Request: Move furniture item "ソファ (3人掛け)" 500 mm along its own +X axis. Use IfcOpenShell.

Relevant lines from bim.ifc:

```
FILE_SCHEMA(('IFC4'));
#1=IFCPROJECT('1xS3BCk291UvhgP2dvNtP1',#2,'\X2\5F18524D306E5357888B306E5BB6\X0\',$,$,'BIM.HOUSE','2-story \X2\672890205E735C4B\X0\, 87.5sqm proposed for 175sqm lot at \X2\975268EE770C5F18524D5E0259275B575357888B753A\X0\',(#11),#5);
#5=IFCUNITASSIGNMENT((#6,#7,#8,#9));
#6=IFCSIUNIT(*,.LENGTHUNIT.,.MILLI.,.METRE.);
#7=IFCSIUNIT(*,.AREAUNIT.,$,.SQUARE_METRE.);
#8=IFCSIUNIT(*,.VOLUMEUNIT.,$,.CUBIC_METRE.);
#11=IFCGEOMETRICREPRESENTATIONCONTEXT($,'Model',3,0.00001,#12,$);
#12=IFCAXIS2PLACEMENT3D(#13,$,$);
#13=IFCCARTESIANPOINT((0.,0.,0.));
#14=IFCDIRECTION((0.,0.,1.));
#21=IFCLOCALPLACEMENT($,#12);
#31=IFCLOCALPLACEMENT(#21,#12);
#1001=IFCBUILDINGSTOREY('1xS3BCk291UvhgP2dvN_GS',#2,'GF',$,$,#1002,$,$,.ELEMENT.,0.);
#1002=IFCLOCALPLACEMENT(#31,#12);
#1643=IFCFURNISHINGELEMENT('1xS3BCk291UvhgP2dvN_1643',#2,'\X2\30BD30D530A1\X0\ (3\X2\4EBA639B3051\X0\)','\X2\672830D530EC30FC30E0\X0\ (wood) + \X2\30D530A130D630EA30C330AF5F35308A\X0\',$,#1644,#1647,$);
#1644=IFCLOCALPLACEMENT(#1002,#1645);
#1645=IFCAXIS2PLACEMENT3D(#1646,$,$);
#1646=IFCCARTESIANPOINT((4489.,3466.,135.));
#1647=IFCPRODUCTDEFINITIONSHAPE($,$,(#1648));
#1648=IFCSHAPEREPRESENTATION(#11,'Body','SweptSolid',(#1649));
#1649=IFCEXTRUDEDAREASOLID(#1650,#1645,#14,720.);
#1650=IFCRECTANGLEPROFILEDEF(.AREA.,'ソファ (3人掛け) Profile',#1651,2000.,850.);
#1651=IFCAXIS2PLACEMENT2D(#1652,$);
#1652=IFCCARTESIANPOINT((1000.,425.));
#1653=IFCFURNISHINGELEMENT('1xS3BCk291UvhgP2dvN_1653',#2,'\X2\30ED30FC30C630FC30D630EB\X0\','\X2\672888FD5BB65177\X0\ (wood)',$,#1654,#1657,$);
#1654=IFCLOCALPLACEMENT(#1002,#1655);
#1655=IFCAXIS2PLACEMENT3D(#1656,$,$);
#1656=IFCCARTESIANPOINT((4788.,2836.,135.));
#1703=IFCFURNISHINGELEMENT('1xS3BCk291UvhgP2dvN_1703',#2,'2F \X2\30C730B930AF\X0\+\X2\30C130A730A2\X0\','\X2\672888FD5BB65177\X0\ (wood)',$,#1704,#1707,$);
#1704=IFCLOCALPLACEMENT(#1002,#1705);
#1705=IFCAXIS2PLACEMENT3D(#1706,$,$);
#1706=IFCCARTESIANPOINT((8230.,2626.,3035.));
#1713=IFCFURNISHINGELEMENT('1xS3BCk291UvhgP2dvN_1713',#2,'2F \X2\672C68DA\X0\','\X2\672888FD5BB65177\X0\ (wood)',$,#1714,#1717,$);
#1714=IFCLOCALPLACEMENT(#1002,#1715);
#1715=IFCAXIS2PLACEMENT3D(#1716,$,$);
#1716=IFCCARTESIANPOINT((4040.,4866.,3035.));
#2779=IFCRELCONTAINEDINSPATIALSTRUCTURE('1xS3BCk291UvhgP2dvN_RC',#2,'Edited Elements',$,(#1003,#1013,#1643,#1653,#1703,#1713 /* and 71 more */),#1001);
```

```python
import ifcopenshell
import ifcopenshell.api.geometry
import ifcopenshell.util.placement

model = ifcopenshell.open("bim.ifc")

item = model.by_guid("1xS3BCk291UvhgP2dvN_1643")
matrix = ifcopenshell.util.placement.get_local_placement(item.ObjectPlacement)
matrix[:3, 3] += matrix[:3, 0] * 500.0
ifcopenshell.api.geometry.edit_object_placement(model, product=item, matrix=matrix, is_si=False)

print(ifcopenshell.util.placement.get_local_placement(item.ObjectPlacement).round(3) + 0.0)

model.write("bim-out.ifc")
```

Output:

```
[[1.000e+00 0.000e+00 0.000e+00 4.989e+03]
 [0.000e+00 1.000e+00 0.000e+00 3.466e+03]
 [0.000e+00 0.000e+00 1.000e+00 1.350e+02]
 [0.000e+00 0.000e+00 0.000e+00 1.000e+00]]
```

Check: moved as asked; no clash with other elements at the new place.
